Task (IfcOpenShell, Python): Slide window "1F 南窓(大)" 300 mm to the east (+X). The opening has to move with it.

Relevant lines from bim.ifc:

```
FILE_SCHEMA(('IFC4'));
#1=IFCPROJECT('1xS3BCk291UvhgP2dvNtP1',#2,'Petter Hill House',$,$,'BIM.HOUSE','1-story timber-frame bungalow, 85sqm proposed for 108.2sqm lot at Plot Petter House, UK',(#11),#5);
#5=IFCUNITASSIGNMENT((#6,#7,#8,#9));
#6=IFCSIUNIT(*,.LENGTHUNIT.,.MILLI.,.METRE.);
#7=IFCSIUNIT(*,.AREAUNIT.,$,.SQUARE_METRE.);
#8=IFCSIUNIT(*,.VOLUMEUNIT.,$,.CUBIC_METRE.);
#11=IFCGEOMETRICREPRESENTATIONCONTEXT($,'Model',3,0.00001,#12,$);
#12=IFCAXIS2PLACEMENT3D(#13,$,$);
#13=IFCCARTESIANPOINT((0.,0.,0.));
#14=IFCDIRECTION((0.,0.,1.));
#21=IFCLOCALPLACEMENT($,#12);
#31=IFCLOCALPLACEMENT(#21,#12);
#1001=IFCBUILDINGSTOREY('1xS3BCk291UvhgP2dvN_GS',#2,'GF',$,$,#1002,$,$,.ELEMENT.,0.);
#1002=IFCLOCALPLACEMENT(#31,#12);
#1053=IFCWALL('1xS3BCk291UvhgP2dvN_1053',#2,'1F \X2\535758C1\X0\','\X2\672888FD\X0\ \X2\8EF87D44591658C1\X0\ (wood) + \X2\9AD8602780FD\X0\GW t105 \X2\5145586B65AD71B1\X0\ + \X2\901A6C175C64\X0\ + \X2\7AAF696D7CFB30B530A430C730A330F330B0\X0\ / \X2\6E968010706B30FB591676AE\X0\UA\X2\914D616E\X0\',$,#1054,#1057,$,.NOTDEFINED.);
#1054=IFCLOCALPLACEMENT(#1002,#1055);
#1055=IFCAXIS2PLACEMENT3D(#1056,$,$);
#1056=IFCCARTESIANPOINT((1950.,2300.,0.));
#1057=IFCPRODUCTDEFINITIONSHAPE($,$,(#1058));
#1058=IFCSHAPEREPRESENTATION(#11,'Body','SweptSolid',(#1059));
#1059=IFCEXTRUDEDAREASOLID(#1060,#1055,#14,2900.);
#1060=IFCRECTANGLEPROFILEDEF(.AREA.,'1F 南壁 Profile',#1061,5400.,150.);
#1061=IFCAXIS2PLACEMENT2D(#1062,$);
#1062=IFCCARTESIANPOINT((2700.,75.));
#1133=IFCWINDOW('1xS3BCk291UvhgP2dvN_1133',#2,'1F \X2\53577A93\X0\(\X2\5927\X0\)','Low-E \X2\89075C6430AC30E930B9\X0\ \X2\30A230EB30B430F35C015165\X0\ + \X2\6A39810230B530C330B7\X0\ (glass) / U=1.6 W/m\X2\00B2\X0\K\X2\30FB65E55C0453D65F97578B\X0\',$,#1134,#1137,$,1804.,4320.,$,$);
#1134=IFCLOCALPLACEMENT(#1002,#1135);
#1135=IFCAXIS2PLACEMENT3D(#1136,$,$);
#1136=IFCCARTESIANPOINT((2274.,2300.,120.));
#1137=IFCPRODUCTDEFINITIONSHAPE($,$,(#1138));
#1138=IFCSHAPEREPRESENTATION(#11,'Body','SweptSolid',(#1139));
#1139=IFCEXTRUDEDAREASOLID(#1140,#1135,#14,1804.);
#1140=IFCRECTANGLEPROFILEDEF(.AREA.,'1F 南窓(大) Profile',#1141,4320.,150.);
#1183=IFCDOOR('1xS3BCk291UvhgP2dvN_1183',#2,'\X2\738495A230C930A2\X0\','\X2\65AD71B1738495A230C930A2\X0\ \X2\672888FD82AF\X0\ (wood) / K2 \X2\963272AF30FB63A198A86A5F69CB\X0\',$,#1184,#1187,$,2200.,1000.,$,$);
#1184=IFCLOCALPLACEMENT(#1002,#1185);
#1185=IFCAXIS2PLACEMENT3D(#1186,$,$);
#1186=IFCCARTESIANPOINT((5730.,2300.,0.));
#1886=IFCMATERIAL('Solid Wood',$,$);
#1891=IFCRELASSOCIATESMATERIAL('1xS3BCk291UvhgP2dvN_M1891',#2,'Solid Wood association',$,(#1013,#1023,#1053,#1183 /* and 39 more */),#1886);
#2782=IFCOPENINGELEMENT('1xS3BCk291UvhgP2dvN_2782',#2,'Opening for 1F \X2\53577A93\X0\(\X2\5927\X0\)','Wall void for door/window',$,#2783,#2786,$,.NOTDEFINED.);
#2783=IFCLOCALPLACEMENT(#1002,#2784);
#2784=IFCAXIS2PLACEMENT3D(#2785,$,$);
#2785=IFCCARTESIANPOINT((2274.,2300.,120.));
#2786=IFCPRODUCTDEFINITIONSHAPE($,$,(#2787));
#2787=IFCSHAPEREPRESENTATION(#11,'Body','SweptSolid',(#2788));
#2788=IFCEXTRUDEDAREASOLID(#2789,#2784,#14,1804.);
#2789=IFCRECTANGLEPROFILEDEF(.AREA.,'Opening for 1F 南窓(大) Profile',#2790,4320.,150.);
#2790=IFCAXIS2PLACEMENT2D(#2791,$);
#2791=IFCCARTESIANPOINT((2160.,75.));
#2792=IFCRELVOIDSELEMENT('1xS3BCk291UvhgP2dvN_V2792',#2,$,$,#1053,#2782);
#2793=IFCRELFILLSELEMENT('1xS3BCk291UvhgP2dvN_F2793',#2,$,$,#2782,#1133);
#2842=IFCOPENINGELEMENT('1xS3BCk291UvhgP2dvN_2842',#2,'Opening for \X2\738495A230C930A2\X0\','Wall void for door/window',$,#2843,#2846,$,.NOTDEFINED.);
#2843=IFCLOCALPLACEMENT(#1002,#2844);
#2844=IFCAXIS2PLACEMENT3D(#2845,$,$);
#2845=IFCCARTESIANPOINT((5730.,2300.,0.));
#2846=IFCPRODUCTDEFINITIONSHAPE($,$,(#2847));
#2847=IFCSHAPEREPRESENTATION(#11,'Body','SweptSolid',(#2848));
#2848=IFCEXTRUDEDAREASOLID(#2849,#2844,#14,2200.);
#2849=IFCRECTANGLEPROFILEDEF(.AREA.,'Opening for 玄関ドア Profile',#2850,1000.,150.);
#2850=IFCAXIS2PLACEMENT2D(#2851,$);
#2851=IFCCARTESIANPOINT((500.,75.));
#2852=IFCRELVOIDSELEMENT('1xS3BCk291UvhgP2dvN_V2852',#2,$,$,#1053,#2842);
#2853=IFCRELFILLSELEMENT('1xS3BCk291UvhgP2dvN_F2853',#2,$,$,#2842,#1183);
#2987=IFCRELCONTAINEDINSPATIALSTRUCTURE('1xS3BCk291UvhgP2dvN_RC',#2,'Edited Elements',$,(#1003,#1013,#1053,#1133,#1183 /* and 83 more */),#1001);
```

```python
import ifcopenshell
import ifcopenshell.api.geometry
import ifcopenshell.util.placement

model = ifcopenshell.open("bim.ifc")

window = model.by_guid("1xS3BCk291UvhgP2dvN_1133")
opening = window.FillsVoids[0].RelatingOpeningElement
wall = opening.VoidsElements[0].RelatingBuildingElement

wall_matrix = ifcopenshell.util.placement.get_local_placement(wall.ObjectPlacement)
shift = wall_matrix[:3, 0] * 300.0
before = ifcopenshell.util.placement.get_local_placement(window.ObjectPlacement)[:3, 3].copy()

# The window is not placed relative to its opening, so move both.
for product in (opening, window):
    matrix = ifcopenshell.util.placement.get_local_placement(product.ObjectPlacement)
    matrix[:3, 3] += shift
    ifcopenshell.api.geometry.edit_object_placement(model, product=product, matrix=matrix, is_si=False)

after = ifcopenshell.util.placement.get_local_placement(window.ObjectPlacement)[:3, 3]
print("window moved by", (after - before).round(3) + 0.0)

model.write("bim_rev.ifc")
```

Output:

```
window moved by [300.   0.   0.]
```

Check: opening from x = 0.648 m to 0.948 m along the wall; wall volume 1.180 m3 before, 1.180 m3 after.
